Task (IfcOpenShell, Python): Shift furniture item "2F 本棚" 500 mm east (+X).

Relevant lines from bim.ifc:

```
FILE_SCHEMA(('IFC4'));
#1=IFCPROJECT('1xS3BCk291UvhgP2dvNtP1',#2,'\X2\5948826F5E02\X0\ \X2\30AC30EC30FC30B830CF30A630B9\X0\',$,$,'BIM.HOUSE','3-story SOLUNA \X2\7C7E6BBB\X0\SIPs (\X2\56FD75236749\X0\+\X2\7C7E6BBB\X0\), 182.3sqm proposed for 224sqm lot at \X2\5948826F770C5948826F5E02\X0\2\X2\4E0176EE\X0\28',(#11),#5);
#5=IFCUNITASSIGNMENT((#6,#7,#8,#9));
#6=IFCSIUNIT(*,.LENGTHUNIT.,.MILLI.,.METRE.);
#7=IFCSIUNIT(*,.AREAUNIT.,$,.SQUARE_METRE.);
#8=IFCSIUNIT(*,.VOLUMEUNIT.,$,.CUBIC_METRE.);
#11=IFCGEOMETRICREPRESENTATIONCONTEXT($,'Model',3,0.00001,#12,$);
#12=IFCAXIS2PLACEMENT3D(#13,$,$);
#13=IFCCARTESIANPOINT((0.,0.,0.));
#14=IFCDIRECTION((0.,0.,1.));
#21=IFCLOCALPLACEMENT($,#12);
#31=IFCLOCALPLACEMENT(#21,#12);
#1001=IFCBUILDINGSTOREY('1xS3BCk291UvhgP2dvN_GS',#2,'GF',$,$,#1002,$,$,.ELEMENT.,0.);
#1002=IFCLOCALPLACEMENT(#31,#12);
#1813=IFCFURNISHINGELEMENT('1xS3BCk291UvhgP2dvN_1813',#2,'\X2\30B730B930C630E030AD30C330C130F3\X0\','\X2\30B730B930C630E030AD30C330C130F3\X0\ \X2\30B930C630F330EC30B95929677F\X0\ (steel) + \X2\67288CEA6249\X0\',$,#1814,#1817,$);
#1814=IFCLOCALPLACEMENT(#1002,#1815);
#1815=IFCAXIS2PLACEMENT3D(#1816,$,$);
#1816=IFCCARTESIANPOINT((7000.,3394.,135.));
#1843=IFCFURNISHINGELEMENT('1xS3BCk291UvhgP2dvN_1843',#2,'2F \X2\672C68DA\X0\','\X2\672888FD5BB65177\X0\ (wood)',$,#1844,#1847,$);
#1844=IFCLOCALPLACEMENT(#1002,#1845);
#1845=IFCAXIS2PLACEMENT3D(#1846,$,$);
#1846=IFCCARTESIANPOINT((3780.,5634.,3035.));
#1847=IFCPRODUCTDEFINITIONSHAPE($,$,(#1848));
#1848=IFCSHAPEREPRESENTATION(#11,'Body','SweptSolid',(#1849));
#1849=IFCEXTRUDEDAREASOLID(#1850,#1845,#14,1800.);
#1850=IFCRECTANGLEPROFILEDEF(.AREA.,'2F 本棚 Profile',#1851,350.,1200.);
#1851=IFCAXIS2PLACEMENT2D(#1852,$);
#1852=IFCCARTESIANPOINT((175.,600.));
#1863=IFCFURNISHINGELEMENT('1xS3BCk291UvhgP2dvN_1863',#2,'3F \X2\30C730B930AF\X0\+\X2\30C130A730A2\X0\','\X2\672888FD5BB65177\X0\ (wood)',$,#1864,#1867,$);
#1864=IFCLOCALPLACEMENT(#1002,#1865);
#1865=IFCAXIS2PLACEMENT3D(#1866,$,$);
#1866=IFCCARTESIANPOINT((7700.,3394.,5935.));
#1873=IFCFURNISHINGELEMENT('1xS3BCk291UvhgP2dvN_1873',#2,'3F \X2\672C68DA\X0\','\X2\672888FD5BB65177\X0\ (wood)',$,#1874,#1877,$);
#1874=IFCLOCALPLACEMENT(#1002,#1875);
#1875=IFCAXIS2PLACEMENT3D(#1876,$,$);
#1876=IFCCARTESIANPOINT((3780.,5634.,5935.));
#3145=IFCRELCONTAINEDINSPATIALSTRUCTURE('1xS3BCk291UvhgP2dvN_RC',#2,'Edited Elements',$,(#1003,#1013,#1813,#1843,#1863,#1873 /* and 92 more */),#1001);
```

```python
import ifcopenshell
import ifcopenshell.api.geometry
import ifcopenshell.util.placement
import ifcopenshell.util.unit

model = ifcopenshell.open("bim.ifc")
unit_scale = ifcopenshell.util.unit.calculate_unit_scale(model)

item = model.by_guid("1xS3BCk291UvhgP2dvN_1843")
matrix = ifcopenshell.util.placement.get_local_placement(item.ObjectPlacement)
matrix[0, 3] += 0.5 / unit_scale
ifcopenshell.api.geometry.edit_object_placement(model, product=item, matrix=matrix, is_si=False)

print(ifcopenshell.util.placement.get_local_placement(item.ObjectPlacement).round(3) + 0.0)

model.write("bim_updated.ifc")
```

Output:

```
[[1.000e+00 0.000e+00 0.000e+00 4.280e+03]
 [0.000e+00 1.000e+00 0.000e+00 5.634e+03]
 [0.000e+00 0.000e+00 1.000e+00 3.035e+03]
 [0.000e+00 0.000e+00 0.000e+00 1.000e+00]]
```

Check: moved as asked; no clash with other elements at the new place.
